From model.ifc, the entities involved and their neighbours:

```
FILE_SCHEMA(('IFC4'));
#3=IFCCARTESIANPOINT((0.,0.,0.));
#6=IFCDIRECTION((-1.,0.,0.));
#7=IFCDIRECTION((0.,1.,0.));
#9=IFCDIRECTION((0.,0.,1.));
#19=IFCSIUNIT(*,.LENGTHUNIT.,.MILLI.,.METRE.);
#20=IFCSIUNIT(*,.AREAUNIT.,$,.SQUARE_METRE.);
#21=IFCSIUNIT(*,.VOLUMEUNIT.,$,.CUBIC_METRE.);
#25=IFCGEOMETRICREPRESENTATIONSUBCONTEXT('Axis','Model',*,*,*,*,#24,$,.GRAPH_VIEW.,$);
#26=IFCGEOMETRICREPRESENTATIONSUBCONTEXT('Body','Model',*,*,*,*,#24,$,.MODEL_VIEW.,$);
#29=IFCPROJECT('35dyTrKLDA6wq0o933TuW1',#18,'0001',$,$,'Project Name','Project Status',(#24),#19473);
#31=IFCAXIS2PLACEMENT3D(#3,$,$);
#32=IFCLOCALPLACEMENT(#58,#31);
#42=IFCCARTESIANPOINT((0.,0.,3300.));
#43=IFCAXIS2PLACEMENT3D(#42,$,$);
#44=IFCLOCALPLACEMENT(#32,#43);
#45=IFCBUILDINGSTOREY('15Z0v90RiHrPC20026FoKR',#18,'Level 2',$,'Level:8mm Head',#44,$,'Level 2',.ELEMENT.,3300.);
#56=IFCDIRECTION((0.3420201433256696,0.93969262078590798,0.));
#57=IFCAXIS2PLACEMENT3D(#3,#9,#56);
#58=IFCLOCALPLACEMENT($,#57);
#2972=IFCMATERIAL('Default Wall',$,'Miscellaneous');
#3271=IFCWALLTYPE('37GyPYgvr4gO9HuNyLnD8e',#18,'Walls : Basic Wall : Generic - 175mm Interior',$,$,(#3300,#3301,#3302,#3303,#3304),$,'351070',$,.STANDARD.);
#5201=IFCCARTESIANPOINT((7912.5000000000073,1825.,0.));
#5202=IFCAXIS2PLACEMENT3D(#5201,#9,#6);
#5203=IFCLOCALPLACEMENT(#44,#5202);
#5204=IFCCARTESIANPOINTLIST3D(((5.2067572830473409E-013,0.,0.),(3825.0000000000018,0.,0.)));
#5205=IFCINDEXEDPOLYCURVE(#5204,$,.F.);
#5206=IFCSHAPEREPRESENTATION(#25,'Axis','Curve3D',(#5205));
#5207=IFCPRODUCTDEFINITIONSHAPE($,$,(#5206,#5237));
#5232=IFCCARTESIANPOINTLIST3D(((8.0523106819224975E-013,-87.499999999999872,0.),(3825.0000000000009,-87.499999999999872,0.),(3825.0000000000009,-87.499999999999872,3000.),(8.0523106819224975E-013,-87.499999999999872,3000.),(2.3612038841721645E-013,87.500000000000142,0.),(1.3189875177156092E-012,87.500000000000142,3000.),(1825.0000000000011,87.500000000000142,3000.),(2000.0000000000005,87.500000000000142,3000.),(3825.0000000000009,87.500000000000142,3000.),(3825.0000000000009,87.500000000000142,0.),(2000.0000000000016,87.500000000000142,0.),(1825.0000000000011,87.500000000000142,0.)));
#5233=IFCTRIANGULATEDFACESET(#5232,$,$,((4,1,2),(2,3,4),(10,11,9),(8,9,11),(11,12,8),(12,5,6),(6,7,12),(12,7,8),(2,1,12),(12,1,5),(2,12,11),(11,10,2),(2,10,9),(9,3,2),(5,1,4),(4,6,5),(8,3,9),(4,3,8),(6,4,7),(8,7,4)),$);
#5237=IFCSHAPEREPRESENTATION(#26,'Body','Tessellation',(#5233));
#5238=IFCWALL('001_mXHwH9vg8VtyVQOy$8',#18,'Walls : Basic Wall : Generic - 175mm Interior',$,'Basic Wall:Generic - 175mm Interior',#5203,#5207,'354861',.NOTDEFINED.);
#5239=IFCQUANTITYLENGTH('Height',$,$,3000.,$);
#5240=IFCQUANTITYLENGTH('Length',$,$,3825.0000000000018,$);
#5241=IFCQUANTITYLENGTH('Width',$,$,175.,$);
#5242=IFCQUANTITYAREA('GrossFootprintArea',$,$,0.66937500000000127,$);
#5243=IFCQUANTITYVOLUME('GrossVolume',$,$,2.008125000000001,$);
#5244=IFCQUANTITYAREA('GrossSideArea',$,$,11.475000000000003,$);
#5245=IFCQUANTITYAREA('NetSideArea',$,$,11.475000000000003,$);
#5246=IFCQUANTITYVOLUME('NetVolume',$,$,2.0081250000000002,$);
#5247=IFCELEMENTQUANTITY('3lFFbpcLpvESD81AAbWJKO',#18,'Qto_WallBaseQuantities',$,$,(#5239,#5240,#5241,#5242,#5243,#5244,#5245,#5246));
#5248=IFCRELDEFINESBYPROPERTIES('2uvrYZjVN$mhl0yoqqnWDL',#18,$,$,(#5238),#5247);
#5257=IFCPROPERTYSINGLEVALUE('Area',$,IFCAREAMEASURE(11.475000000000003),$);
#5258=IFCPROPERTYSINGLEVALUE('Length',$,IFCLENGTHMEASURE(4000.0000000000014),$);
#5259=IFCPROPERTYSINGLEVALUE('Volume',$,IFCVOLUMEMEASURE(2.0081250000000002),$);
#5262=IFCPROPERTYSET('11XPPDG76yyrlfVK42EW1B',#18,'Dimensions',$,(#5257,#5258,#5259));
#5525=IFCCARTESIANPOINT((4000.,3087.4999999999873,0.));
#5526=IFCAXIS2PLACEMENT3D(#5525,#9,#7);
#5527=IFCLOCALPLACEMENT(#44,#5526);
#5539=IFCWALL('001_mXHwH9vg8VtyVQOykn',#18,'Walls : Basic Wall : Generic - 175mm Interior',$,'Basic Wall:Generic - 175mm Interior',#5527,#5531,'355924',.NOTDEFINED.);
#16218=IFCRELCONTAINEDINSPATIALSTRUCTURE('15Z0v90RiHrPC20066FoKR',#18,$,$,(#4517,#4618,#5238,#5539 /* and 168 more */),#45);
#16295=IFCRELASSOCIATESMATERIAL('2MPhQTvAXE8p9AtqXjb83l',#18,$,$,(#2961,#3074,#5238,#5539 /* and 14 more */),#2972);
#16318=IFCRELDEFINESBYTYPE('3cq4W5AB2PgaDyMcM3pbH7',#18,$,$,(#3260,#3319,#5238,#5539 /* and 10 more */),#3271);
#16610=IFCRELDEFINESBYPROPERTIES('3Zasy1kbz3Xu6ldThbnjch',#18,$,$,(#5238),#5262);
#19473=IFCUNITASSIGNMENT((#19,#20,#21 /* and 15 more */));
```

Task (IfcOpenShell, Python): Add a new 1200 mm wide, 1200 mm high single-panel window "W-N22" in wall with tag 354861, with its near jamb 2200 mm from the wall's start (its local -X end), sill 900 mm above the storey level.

```python
import numpy as np
import ifcopenshell
import ifcopenshell.api.feature
import ifcopenshell.api.geometry
import ifcopenshell.api.pset
import ifcopenshell.api.root
import ifcopenshell.api.spatial
import ifcopenshell.geom
import ifcopenshell.util.element
import ifcopenshell.util.placement
import ifcopenshell.util.representation
import ifcopenshell.util.shape
import ifcopenshell.util.unit

model = ifcopenshell.open("model.ifc")
unit_scale = ifcopenshell.util.unit.calculate_unit_scale(model)
area_scale = ifcopenshell.util.unit.calculate_unit_scale(model, "AREAUNIT")
volume_scale = ifcopenshell.util.unit.calculate_unit_scale(model, "VOLUMEUNIT")
settings = ifcopenshell.geom.settings()


def volume(element):
    """Net volume in cubic metres, openings subtracted."""
    shape = ifcopenshell.geom.create_shape(settings, element)
    return ifcopenshell.util.shape.get_volume(shape.geometry)


wall = model.by_id(5238)
storey = ifcopenshell.util.element.get_container(wall, ifc_class="IfcBuildingStorey")
context = ifcopenshell.util.representation.get_context(model, "Model", "Body", "MODEL_VIEW")
before = volume(wall)

width, height, from_end, sill = 1.2, 1.2, 2.2, 0.9  # metres

# The wall runs along its own X axis, and the end named is its -X end.
wall_shape = ifcopenshell.geom.create_shape(settings, wall)
x, y, z = ifcopenshell.util.shape.get_vertices(wall_shape.geometry).T
start = x.min() + from_end
face, thickness = float(y.min()), float(y.max() - y.min())
wall_matrix = ifcopenshell.util.placement.get_local_placement(wall.ObjectPlacement)
level = ifcopenshell.util.placement.get_local_placement(storey.ObjectPlacement)[2, 3]


def in_wall(x, y):
    """Placement at x, y metres in the wall's axes, at sill height."""
    matrix = wall_matrix.copy()
    matrix[:, 3] = wall_matrix @ np.array([x / unit_scale, y / unit_scale, 0.0, 1.0])
    matrix[2, 3] = level + sill / unit_scale
    return matrix


# Opening: a box that overshoots both wall faces by 50 mm.
opening = ifcopenshell.api.root.create_entity(model, ifc_class="IfcOpeningElement", predefined_type="OPENING")
box = ifcopenshell.api.geometry.add_wall_representation(
    model, context=context, length=width, height=height, thickness=thickness + 0.1
)
ifcopenshell.api.geometry.assign_representation(model, product=opening, representation=box)
ifcopenshell.api.geometry.edit_object_placement(model, product=opening, matrix=in_wall(start, face - 0.05), is_si=False)
ifcopenshell.api.feature.add_feature(model, feature=opening, element=wall)

window = ifcopenshell.api.root.create_entity(model, ifc_class="IfcWindow", name="W-N22", predefined_type="WINDOW")
window.OverallWidth, window.OverallHeight = width / unit_scale, height / unit_scale
window.PartitioningType = "SINGLE_PANEL"
body = ifcopenshell.api.geometry.add_window_representation(
    model,
    context=context,
    overall_width=window.OverallWidth,
    overall_height=window.OverallHeight,
    partition_type="SINGLE_PANEL",
)
ifcopenshell.api.geometry.assign_representation(model, product=window, representation=body)
ifcopenshell.api.spatial.assign_container(model, products=[window], relating_structure=storey)
ifcopenshell.api.feature.add_filling(model, opening=opening, element=window)

# Centre the window in the wall's thickness.
ifcopenshell.api.geometry.edit_object_placement(model, product=window, matrix=in_wall(start, face), is_si=False)
window_shape = ifcopenshell.geom.create_shape(settings, window)
depth = ifcopenshell.util.shape.get_vertices(window_shape.geometry)[:, 1]
offset = face + thickness / 2 - (depth.min() + depth.max()) / 2
ifcopenshell.api.geometry.edit_object_placement(model, product=window, matrix=in_wall(start, offset), is_si=False)

after = volume(wall)

# Update the wall's stored quantities.
qto = model.by_id(ifcopenshell.util.element.get_pset(wall, "Qto_WallBaseQuantities", should_inherit=False)["id"])
ifcopenshell.api.pset.edit_qto(model, qto=qto, properties={
    "NetSideArea": after / thickness / area_scale,
    "NetVolume": after / volume_scale,
})
pset = model.by_id(ifcopenshell.util.element.get_pset(wall, "Dimensions", should_inherit=False)["id"])
ifcopenshell.api.pset.edit_pset(model, pset=pset, properties={
    "Area": model.create_entity("IfcAreaMeasure", after / thickness / area_scale),
    "Volume": model.create_entity("IfcVolumeMeasure", after / volume_scale),
})

print(f"wall volume {before:.3f} -> {after:.3f} m3")

model.write("model_updated.ifc")
```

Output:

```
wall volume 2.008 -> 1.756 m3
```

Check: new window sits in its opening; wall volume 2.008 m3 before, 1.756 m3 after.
